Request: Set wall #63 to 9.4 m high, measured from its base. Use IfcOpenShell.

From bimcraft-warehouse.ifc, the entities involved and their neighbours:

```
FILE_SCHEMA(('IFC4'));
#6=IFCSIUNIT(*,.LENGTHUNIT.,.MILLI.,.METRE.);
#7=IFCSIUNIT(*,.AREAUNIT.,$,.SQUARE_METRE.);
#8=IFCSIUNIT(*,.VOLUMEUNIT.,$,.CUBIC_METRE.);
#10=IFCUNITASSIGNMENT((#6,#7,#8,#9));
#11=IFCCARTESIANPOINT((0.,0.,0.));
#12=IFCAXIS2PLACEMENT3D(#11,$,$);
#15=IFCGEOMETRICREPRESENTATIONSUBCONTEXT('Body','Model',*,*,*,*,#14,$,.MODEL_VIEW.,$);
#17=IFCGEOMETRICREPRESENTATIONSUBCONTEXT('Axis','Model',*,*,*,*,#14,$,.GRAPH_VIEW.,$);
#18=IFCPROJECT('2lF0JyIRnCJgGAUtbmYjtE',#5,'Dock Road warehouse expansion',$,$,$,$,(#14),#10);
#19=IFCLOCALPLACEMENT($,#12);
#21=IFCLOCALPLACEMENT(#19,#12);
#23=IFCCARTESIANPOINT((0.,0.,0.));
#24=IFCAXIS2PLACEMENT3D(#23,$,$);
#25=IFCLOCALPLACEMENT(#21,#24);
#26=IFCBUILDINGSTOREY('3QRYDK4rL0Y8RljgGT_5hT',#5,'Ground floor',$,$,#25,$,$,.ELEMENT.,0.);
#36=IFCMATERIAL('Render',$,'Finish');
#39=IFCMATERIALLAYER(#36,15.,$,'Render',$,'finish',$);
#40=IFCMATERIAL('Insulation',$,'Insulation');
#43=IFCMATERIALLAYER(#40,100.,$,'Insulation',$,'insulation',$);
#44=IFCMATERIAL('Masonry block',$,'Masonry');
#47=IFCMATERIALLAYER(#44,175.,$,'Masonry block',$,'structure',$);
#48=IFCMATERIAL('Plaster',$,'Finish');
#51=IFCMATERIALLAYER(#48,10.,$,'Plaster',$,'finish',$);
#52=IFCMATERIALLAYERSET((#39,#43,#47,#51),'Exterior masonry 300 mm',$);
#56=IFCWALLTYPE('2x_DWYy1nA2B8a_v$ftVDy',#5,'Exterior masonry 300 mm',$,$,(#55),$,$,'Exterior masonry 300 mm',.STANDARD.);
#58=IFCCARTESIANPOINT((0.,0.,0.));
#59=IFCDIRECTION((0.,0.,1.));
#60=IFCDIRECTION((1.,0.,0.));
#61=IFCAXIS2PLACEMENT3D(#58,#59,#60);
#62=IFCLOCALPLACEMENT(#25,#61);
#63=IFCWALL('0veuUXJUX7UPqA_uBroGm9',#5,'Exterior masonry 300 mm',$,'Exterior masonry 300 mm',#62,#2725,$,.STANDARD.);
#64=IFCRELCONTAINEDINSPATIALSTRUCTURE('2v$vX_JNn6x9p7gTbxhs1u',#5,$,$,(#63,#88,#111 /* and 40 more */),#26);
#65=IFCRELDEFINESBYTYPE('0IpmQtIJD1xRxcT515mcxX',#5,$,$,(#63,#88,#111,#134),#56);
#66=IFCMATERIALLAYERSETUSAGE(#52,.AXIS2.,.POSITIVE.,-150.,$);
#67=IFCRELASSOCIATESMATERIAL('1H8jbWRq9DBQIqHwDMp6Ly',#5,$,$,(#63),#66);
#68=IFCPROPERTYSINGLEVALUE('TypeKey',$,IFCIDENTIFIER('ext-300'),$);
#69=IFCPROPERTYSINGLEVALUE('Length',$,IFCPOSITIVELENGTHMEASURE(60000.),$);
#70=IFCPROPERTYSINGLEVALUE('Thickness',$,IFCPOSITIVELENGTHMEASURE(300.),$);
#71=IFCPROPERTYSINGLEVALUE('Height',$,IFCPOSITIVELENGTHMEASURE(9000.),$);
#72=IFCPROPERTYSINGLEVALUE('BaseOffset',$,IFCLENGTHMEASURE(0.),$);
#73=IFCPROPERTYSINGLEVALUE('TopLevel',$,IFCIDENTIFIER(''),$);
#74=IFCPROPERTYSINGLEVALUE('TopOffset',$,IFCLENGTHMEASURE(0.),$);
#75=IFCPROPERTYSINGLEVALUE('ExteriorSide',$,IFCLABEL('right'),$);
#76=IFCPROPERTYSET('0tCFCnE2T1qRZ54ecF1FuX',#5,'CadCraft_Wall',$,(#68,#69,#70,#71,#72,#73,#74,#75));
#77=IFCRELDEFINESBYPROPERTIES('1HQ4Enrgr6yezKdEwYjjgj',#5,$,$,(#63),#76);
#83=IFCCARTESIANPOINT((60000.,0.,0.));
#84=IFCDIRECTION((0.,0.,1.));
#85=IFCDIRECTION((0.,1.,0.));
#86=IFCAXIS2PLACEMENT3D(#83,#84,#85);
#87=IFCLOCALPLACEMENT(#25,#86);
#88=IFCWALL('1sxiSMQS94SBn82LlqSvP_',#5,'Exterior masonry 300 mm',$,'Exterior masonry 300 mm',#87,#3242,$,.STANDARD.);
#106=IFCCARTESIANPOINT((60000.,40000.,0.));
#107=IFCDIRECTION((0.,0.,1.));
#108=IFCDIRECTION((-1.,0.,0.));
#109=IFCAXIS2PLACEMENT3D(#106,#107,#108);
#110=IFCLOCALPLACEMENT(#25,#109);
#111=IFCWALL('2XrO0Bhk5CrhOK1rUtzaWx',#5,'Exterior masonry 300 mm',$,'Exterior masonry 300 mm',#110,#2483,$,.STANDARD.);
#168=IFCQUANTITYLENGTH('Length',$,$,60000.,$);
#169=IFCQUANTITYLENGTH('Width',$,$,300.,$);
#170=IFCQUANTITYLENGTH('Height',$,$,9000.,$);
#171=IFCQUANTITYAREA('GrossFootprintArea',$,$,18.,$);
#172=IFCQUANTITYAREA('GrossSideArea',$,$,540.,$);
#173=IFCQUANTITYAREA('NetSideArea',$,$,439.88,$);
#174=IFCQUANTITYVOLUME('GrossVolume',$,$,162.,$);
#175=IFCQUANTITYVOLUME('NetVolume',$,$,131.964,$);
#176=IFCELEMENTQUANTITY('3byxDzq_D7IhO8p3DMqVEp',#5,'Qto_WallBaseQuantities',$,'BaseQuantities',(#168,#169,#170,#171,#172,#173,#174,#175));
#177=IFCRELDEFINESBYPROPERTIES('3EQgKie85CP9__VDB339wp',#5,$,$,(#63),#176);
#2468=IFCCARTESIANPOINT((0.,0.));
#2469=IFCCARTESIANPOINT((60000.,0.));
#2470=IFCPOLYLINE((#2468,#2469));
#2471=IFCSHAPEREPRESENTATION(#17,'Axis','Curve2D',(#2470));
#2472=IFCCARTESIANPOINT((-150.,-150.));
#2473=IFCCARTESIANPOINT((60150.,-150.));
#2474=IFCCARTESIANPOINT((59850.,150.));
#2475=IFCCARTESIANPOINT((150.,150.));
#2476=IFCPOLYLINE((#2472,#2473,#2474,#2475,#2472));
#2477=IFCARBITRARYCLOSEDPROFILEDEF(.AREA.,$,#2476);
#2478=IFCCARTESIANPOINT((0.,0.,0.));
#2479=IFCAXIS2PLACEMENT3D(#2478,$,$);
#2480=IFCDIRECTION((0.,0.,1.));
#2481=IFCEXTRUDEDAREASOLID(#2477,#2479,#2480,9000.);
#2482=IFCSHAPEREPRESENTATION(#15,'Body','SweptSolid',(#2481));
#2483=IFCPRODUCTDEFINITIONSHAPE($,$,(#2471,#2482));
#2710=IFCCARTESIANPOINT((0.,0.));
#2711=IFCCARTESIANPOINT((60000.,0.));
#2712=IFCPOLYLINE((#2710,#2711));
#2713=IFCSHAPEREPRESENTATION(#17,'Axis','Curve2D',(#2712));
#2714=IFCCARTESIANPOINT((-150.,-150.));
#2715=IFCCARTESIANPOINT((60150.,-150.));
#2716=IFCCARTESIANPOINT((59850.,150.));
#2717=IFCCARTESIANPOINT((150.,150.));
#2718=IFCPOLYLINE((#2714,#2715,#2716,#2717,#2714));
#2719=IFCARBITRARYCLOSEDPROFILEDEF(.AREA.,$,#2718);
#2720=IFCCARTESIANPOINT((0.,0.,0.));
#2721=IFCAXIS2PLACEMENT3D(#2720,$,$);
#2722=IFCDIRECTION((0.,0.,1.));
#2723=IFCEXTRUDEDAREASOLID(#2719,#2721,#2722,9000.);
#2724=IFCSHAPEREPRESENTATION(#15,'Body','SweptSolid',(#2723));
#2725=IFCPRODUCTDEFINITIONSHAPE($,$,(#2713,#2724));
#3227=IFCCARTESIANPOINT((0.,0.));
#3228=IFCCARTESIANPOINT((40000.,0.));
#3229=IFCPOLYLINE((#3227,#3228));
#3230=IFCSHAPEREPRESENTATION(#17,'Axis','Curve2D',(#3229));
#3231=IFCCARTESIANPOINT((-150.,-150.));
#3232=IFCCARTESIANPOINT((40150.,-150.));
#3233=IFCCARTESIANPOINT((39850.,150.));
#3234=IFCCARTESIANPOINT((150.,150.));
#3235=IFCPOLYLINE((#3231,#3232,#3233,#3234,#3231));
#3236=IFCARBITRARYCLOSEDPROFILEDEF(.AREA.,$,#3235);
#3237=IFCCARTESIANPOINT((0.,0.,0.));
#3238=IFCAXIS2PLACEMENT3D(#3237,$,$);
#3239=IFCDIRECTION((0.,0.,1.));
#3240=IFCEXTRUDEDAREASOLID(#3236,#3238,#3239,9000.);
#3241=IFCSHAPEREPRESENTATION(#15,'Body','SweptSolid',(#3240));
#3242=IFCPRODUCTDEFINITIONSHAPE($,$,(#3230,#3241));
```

```python
import ifcopenshell
import ifcopenshell.api.pset
import ifcopenshell.geom
import ifcopenshell.util.element
import ifcopenshell.util.representation
import ifcopenshell.util.shape
import ifcopenshell.util.unit

model = ifcopenshell.open("bimcraft-warehouse.ifc")
unit_scale = ifcopenshell.util.unit.calculate_unit_scale(model)
area_scale = ifcopenshell.util.unit.calculate_unit_scale(model, "AREAUNIT")
volume_scale = ifcopenshell.util.unit.calculate_unit_scale(model, "VOLUMEUNIT")
settings = ifcopenshell.geom.settings()


def volume(element):
    """Net volume in cubic metres, openings subtracted."""
    shape = ifcopenshell.geom.create_shape(settings, element)
    return ifcopenshell.util.shape.get_volume(shape.geometry)


wall = model.by_guid("0veuUXJUX7UPqA_uBroGm9")
before = volume(wall)

body = ifcopenshell.util.representation.get_representation(wall, "Model", "Body")
solid = body.Items[0]
old_height = solid.Depth
solid.Depth = 9400.0
after = volume(wall)
thickness = 0.3  # wall thickness in metres

# Update the stored height, areas and volumes.
pset = model.by_id(ifcopenshell.util.element.get_pset(wall, "CadCraft_Wall", should_inherit=False)["id"])
ifcopenshell.api.pset.edit_pset(model, pset=pset, properties={
    "Height": model.create_entity("IfcPositiveLengthMeasure", solid.Depth),
})
qto = model.by_id(ifcopenshell.util.element.get_pset(wall, "Qto_WallBaseQuantities", should_inherit=False)["id"])
ifcopenshell.api.pset.edit_qto(model, qto=qto, properties={
    "Height": solid.Depth,
    "GrossSideArea": ifcopenshell.util.element.get_pset(wall, "Qto_WallBaseQuantities", "GrossSideArea") * solid.Depth / old_height,
    "NetSideArea": after / thickness / area_scale,
    "GrossVolume": ifcopenshell.util.element.get_pset(wall, "Qto_WallBaseQuantities", "GrossVolume") * solid.Depth / old_height,
    "NetVolume": after / volume_scale,
})

print(f"height {old_height:g} -> {solid.Depth:g}, volume {before:.3f} -> {after:.3f} m3")

model.write("bimcraft-warehouse-out.ifc")
```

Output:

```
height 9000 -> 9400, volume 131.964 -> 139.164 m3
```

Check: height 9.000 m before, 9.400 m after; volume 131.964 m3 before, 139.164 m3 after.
